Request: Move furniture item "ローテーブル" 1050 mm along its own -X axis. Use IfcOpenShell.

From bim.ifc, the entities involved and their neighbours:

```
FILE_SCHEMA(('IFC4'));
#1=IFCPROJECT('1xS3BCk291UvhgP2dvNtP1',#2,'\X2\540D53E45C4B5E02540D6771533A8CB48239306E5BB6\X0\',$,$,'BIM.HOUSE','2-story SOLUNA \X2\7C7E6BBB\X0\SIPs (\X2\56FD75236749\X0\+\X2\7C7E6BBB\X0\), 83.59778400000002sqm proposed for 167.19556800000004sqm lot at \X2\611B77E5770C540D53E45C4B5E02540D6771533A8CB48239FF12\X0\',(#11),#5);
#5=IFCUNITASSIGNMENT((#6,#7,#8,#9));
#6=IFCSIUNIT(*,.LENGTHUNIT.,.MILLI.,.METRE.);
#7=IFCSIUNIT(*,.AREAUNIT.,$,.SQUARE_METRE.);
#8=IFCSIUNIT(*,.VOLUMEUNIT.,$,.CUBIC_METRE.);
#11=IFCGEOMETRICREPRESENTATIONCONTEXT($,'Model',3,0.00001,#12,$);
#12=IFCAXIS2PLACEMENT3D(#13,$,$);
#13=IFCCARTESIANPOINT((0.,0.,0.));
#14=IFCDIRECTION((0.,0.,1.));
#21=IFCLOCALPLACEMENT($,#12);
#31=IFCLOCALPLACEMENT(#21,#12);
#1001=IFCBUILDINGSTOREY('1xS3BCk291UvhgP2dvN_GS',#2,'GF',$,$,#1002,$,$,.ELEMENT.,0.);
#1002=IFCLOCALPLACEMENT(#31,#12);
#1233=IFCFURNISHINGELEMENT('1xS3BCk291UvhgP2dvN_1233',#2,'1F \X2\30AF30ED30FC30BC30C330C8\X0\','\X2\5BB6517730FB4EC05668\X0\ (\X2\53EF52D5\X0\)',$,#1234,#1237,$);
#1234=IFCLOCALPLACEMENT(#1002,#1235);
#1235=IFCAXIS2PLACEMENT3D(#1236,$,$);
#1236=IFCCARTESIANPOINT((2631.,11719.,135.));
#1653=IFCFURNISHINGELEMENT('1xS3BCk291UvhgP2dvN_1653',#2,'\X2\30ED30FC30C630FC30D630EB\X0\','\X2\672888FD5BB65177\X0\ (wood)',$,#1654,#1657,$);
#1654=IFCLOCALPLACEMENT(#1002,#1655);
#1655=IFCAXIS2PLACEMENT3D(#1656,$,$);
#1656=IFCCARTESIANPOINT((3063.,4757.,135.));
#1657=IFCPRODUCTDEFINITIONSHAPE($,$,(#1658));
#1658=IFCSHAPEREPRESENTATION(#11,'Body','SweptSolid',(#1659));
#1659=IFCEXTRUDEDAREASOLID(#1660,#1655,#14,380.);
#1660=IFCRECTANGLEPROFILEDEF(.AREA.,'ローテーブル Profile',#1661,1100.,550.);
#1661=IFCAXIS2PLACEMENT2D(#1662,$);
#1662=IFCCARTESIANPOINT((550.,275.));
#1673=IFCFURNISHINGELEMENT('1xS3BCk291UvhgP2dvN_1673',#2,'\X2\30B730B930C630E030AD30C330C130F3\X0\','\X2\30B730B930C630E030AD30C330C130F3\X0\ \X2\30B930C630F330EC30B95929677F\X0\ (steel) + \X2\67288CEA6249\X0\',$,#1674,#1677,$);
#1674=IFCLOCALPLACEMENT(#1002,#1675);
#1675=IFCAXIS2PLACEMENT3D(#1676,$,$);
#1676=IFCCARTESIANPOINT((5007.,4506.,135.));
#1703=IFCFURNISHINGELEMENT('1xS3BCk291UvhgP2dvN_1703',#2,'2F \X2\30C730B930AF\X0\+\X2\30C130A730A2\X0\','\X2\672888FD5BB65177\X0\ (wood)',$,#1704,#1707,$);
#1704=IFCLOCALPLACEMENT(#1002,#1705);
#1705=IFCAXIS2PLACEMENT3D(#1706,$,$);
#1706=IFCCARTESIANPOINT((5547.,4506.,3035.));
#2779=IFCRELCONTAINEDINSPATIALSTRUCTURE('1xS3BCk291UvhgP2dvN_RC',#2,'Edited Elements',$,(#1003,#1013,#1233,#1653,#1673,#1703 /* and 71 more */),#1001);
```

```python
import ifcopenshell
import ifcopenshell.api.geometry
import ifcopenshell.util.placement
import ifcopenshell.util.unit

model = ifcopenshell.open("bim.ifc")
unit_scale = ifcopenshell.util.unit.calculate_unit_scale(model)

item = model.by_id(1653)
matrix = ifcopenshell.util.placement.get_local_placement(item.ObjectPlacement)
matrix[:3, 3] -= matrix[:3, 0] * 1.05 / unit_scale
ifcopenshell.api.geometry.edit_object_placement(model, product=item, matrix=matrix, is_si=False)

print(ifcopenshell.util.placement.get_local_placement(item.ObjectPlacement).round(3) + 0.0)

model.write("bim_rev.ifc")
```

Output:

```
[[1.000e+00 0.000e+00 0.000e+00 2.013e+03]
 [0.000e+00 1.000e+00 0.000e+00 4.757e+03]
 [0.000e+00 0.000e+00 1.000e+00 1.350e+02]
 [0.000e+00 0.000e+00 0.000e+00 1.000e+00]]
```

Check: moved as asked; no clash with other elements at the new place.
